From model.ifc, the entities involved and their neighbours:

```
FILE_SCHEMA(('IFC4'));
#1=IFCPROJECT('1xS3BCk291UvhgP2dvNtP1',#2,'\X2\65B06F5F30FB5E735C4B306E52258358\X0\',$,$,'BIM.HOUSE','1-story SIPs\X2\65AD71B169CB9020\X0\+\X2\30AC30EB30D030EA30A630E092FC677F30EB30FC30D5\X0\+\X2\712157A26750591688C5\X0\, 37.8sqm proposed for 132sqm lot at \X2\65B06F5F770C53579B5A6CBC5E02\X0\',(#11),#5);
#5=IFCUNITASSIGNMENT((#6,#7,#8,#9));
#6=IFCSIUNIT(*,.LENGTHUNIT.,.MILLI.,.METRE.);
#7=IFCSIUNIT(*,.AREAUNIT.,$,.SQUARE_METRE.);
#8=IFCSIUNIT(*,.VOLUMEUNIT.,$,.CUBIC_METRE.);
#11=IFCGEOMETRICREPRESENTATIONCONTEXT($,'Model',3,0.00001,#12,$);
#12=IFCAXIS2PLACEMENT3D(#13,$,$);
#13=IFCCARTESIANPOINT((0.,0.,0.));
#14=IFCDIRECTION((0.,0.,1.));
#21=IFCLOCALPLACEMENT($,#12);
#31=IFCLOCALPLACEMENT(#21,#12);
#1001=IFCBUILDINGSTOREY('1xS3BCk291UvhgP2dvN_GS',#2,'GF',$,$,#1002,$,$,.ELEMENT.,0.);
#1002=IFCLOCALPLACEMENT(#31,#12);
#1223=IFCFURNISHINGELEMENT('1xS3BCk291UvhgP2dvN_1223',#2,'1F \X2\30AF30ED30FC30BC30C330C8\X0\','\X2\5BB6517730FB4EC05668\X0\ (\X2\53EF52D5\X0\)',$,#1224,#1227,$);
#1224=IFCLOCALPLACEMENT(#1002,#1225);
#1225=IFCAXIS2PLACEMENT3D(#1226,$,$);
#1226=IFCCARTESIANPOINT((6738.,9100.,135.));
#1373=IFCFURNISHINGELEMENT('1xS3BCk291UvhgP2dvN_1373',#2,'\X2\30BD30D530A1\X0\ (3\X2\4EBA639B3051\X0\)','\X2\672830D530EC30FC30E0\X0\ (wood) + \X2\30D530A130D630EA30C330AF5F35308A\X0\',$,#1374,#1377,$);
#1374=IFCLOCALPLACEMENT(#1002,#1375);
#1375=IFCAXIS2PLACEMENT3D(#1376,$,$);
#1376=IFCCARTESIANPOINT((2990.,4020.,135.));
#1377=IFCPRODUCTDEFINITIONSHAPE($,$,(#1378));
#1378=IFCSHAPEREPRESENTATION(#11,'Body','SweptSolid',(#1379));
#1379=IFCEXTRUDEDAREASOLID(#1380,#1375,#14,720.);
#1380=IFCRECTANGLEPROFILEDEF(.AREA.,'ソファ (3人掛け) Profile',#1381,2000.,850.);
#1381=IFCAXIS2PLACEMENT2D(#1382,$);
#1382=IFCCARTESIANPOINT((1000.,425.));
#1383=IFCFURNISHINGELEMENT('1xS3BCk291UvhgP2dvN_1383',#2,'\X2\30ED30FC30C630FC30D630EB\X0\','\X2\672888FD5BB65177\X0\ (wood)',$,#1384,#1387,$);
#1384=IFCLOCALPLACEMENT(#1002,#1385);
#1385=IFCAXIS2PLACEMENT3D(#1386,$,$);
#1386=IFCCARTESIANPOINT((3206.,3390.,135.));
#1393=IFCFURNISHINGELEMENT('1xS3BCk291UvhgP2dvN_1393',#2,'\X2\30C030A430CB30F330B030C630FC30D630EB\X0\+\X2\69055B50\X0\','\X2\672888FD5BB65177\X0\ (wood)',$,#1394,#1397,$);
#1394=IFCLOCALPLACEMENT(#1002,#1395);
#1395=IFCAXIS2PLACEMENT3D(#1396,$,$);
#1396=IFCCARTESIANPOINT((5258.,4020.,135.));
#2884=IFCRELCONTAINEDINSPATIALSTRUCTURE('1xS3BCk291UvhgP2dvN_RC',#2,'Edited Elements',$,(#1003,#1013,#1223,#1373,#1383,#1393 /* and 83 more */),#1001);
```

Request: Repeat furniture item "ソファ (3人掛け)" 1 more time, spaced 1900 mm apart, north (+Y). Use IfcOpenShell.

```python
import numpy as np
import ifcopenshell
import ifcopenshell.api.geometry
import ifcopenshell.api.root
import ifcopenshell.util.element
import ifcopenshell.util.placement
import ifcopenshell.util.unit

model = ifcopenshell.open("model.ifc")
unit_scale = ifcopenshell.util.unit.calculate_unit_scale(model)


def reuse_history(source, copy):
    """copy_class also copies each property set's owner history, people and application; keep the originals."""
    for rel in copy.IsDefinedBy:
        if rel.is_a("IfcRelDefinesByProperties") and (history := rel.RelatingPropertyDefinition.OwnerHistory):
            rel.RelatingPropertyDefinition.OwnerHistory = source.OwnerHistory
            ifcopenshell.util.element.remove_deep2(model, history)


source = model.by_guid("1xS3BCk291UvhgP2dvN_1373")
base = ifcopenshell.util.placement.get_local_placement(source.ObjectPlacement)
step = np.array([0.0, 1.0, 0.0]) * 1.9 / unit_scale

for i in range(1, 2):
    copy = ifcopenshell.api.root.copy_class(model, product=source)
    copy.Representation = ifcopenshell.util.element.copy_deep(
        model, source.Representation, exclude=["IfcGeometricRepresentationContext", "IfcRepresentationMap"]
    )
    reuse_history(source, copy)
    matrix = base.copy()
    matrix[:3, 3] += i * step
    print("added at", matrix[:3, 3].round(3) + 0.0)
    ifcopenshell.api.geometry.edit_object_placement(model, product=copy, matrix=matrix, is_si=False)

model.write("model_rev.ifc")
```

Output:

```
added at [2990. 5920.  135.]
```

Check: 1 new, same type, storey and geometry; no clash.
